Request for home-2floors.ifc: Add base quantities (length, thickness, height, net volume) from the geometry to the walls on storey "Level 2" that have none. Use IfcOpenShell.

First a look at what the model holds.

```python
import ifcopenshell
import ifcopenshell.util.element
import ifcopenshell.util.unit

model = ifcopenshell.open("home-2floors.ifc")
print(model.schema)
for unit_type in ("LENGTHUNIT", "AREAUNIT", "VOLUMEUNIT"):
    print(unit_type, ifcopenshell.util.unit.calculate_unit_scale(model, unit_type))
storey = next(s for s in model.by_type("IfcBuildingStorey") if s.Name == "Level 2")
walls = [e for e in ifcopenshell.util.element.get_decomposition(storey) if e.is_a("IfcWall")]
for e in sorted(walls, key=lambda e: e.id()):
    print(e.id(), e.is_a(), e.Name, list(ifcopenshell.util.element.get_psets(e, qtos_only=True)), sep=" | ")
```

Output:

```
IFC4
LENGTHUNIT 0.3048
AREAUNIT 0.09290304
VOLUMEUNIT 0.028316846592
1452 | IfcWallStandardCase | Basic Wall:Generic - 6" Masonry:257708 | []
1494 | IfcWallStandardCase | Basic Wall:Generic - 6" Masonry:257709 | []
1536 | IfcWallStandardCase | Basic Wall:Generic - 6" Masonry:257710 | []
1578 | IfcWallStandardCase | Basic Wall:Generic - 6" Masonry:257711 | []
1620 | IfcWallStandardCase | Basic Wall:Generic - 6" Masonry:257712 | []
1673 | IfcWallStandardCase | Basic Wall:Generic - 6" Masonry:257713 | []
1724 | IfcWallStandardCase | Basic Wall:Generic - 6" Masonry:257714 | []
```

```python
import ifcopenshell
import ifcopenshell.api.pset
import ifcopenshell.geom
import ifcopenshell.util.element
import ifcopenshell.util.shape
import ifcopenshell.util.unit

model = ifcopenshell.open("home-2floors.ifc")
unit_scale = ifcopenshell.util.unit.calculate_unit_scale(model)
volume_scale = ifcopenshell.util.unit.calculate_unit_scale(model, "VOLUMEUNIT")
settings = ifcopenshell.geom.settings()

storey = next(s for s in model.by_type("IfcBuildingStorey") if s.Name == "Level 2")
walls = [e for e in ifcopenshell.util.element.get_decomposition(storey) if e.is_a("IfcWall")]

for e in sorted(walls, key=lambda e: e.id()):
    if ifcopenshell.util.element.get_psets(e, qtos_only=True, should_inherit=False):
        continue
    # Geometry comes back in metres, in the element's own axes.
    shape = ifcopenshell.geom.create_shape(settings, e)
    values = {
        "Length": ifcopenshell.util.shape.get_x(shape.geometry) / unit_scale,
        "Width": ifcopenshell.util.shape.get_y(shape.geometry) / unit_scale,
        "Height": ifcopenshell.util.shape.get_z(shape.geometry) / unit_scale,
        "NetVolume": ifcopenshell.util.shape.get_volume(shape.geometry) / volume_scale,
    }
    qto = ifcopenshell.api.pset.add_qto(model, product=e, name="Qto_WallBaseQuantities")
    ifcopenshell.api.pset.edit_qto(model, qto=qto, properties=values)
    print(e.id(), {k: round(v, 3) for k, v in values.items()})

model.write("home-2floors-out.ifc")
```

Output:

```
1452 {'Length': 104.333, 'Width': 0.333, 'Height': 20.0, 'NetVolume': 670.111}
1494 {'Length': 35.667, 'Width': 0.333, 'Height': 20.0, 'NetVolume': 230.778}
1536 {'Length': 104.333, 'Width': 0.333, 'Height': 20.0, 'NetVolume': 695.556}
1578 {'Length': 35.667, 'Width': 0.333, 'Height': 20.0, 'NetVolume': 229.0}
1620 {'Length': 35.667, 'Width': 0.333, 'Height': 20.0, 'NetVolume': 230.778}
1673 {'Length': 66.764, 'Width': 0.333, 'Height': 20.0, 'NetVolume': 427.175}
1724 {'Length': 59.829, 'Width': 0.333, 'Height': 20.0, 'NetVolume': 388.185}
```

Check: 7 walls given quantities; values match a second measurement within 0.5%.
